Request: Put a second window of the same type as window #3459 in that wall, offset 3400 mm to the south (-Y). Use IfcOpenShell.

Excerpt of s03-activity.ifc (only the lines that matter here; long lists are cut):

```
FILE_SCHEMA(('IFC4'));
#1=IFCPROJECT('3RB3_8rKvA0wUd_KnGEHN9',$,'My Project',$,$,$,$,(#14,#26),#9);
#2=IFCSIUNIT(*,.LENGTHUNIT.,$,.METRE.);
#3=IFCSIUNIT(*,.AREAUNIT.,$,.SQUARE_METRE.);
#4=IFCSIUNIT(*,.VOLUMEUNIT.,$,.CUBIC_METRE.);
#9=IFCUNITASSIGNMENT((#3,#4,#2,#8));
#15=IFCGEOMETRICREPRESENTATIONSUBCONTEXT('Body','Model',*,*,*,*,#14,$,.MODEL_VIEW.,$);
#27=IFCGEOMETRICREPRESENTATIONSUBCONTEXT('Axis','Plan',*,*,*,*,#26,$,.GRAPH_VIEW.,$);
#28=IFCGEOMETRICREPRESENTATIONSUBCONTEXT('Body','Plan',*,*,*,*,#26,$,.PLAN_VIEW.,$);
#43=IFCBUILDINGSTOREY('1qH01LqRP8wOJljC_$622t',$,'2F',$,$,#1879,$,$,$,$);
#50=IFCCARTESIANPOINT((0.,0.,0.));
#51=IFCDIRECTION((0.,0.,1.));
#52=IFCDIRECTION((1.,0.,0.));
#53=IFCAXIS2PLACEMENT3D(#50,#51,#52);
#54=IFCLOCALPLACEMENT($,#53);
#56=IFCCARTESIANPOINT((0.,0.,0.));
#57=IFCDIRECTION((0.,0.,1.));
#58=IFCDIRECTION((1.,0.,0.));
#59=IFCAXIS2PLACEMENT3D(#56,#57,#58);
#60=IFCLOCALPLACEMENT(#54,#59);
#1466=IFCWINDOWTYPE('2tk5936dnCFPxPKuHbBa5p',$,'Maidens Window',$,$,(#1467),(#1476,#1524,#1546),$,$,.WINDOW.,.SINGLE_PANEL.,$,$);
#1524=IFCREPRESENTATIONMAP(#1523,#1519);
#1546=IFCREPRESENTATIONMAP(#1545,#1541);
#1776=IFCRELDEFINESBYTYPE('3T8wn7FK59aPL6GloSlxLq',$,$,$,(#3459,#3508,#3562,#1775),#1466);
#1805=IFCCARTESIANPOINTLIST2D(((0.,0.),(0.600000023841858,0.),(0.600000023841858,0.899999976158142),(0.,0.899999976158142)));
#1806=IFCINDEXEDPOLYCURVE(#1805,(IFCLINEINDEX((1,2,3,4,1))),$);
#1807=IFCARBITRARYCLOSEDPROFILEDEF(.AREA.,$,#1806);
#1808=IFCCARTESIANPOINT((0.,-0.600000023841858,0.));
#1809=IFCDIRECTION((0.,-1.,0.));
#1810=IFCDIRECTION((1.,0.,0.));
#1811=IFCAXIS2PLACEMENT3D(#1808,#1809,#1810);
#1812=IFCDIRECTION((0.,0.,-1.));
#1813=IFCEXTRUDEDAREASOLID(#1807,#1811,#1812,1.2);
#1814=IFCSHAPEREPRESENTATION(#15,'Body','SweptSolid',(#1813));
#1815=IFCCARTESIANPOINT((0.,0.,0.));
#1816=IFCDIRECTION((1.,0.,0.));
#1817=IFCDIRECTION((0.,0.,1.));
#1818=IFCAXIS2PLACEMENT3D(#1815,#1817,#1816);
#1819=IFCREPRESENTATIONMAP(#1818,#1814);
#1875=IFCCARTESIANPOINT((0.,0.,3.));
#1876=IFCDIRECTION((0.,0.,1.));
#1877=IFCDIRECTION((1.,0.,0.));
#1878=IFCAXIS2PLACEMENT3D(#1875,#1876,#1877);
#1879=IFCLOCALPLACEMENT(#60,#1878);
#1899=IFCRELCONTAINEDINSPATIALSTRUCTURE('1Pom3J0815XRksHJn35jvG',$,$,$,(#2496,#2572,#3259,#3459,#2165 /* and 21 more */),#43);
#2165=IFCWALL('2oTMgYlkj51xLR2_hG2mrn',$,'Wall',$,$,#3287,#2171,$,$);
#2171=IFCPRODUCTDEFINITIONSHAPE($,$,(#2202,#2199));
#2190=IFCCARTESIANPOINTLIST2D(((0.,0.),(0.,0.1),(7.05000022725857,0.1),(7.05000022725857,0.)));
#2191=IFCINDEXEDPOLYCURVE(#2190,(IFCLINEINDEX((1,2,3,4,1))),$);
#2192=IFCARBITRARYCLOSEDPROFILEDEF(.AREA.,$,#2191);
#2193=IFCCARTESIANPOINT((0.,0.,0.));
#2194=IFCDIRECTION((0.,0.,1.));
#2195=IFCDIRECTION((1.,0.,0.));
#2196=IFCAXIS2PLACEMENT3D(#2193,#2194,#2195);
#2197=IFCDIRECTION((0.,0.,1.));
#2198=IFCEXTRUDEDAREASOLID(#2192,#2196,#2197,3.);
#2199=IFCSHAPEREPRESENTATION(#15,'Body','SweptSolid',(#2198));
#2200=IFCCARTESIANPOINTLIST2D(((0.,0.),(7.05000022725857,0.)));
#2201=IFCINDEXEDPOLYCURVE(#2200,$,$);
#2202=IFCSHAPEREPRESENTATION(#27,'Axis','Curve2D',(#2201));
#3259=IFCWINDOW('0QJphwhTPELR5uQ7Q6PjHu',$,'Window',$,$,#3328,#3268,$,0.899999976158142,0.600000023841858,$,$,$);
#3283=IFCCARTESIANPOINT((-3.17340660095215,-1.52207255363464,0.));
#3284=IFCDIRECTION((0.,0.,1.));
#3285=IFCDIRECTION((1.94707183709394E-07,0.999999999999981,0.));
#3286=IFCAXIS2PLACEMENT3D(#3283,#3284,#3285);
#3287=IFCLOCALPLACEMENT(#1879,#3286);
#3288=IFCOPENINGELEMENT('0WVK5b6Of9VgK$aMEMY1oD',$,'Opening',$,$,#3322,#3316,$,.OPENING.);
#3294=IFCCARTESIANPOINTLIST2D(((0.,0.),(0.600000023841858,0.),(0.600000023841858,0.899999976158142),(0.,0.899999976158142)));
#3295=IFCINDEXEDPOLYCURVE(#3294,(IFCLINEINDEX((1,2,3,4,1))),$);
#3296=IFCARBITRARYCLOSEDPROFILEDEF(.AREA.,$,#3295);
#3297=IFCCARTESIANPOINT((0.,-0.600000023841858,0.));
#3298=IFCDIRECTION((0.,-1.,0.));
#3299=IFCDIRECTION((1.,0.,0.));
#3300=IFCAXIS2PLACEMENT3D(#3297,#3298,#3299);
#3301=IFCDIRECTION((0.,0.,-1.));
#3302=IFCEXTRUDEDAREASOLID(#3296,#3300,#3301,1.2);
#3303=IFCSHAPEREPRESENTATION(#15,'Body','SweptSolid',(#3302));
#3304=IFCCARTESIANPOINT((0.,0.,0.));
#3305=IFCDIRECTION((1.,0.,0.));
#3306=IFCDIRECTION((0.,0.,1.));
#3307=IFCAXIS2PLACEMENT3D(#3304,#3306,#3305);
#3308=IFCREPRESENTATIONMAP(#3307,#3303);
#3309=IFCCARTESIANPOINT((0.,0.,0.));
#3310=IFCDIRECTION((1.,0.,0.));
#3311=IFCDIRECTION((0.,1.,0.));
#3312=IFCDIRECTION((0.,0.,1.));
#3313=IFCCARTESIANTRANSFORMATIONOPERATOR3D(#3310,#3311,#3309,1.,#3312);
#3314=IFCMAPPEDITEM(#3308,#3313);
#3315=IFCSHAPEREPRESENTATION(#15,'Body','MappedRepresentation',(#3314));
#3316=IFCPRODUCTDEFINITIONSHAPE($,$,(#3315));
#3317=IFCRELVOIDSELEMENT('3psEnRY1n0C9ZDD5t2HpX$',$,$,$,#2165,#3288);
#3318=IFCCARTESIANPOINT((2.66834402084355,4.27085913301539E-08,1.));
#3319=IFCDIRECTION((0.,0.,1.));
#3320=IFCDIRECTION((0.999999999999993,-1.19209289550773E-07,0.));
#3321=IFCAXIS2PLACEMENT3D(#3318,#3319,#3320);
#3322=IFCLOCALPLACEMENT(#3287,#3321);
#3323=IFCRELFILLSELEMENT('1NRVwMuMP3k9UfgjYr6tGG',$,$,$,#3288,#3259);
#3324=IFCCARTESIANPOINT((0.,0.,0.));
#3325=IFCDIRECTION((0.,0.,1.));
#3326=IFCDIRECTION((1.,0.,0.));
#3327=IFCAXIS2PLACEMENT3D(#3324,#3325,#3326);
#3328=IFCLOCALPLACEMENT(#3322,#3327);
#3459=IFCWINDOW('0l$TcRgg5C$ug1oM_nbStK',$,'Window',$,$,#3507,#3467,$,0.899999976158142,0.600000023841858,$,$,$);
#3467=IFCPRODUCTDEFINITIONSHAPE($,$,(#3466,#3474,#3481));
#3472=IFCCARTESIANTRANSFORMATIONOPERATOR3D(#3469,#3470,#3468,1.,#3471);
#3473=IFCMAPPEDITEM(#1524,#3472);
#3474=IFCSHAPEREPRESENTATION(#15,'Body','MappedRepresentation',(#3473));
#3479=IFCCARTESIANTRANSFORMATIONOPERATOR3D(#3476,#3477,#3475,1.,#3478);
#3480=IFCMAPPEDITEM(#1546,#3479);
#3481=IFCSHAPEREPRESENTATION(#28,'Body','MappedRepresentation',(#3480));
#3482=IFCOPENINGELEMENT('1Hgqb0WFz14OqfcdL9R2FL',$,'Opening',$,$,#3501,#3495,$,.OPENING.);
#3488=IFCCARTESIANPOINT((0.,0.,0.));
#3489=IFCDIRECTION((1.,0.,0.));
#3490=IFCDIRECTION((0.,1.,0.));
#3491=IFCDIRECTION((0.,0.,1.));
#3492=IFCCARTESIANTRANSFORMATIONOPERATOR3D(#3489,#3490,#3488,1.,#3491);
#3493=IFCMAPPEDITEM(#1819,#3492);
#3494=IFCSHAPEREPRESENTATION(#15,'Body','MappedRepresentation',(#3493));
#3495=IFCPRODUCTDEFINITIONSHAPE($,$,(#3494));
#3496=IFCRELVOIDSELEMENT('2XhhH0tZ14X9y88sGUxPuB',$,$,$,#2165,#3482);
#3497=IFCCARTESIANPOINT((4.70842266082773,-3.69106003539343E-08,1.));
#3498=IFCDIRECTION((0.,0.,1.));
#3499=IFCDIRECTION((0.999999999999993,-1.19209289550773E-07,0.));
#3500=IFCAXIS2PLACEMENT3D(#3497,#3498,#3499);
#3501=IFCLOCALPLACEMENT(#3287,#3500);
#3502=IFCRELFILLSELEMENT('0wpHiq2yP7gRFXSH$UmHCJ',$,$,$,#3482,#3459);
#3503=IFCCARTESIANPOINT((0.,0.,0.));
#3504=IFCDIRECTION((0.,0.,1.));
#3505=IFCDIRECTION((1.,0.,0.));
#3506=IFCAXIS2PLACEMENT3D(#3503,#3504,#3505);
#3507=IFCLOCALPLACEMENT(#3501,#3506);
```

```python
import ifcopenshell
import ifcopenshell.api.feature
import ifcopenshell.api.geometry
import ifcopenshell.api.root
import ifcopenshell.geom
import ifcopenshell.util.element
import ifcopenshell.util.placement
import ifcopenshell.util.shape
import ifcopenshell.util.unit

model = ifcopenshell.open("s03-activity.ifc")
unit_scale = ifcopenshell.util.unit.calculate_unit_scale(model)
settings = ifcopenshell.geom.settings()


def volume(element):
    """Net volume in cubic metres, openings subtracted."""
    shape = ifcopenshell.geom.create_shape(settings, element)
    return ifcopenshell.util.shape.get_volume(shape.geometry)


window = model.by_guid("0l$TcRgg5C$ug1oM_nbStK")
opening = window.FillsVoids[0].RelatingOpeningElement
wall = opening.VoidsElements[0].RelatingBuildingElement
before = volume(wall)
shift = ifcopenshell.util.placement.get_local_placement(wall.ObjectPlacement)[:3, 0] * -3.4 / unit_scale

# copy_class copies the void relationship, type, container and properties, but no geometry.
new_opening = ifcopenshell.api.root.copy_class(model, product=opening)
new_opening.Representation = ifcopenshell.util.element.copy_deep(
    model, opening.Representation, exclude=["IfcGeometricRepresentationContext", "IfcRepresentationMap"]
)
new_window = ifcopenshell.api.root.copy_class(model, product=window)
new_window.Representation = ifcopenshell.util.element.copy_deep(
    model, window.Representation, exclude=["IfcGeometricRepresentationContext", "IfcRepresentationMap"]
)
ifcopenshell.api.feature.add_filling(model, opening=new_opening, element=new_window)

for old, new in ((opening, new_opening), (window, new_window)):
    matrix = ifcopenshell.util.placement.get_local_placement(old.ObjectPlacement)
    matrix[:3, 3] += shift
    ifcopenshell.api.geometry.edit_object_placement(model, product=new, matrix=matrix, is_si=False)

after = volume(wall)

print(f"wall volume {before:.3f} -> {after:.3f} m3")

model.write("s03-activity_updated.ifc")
```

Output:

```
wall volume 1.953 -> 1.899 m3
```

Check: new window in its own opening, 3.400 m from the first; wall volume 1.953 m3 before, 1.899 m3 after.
